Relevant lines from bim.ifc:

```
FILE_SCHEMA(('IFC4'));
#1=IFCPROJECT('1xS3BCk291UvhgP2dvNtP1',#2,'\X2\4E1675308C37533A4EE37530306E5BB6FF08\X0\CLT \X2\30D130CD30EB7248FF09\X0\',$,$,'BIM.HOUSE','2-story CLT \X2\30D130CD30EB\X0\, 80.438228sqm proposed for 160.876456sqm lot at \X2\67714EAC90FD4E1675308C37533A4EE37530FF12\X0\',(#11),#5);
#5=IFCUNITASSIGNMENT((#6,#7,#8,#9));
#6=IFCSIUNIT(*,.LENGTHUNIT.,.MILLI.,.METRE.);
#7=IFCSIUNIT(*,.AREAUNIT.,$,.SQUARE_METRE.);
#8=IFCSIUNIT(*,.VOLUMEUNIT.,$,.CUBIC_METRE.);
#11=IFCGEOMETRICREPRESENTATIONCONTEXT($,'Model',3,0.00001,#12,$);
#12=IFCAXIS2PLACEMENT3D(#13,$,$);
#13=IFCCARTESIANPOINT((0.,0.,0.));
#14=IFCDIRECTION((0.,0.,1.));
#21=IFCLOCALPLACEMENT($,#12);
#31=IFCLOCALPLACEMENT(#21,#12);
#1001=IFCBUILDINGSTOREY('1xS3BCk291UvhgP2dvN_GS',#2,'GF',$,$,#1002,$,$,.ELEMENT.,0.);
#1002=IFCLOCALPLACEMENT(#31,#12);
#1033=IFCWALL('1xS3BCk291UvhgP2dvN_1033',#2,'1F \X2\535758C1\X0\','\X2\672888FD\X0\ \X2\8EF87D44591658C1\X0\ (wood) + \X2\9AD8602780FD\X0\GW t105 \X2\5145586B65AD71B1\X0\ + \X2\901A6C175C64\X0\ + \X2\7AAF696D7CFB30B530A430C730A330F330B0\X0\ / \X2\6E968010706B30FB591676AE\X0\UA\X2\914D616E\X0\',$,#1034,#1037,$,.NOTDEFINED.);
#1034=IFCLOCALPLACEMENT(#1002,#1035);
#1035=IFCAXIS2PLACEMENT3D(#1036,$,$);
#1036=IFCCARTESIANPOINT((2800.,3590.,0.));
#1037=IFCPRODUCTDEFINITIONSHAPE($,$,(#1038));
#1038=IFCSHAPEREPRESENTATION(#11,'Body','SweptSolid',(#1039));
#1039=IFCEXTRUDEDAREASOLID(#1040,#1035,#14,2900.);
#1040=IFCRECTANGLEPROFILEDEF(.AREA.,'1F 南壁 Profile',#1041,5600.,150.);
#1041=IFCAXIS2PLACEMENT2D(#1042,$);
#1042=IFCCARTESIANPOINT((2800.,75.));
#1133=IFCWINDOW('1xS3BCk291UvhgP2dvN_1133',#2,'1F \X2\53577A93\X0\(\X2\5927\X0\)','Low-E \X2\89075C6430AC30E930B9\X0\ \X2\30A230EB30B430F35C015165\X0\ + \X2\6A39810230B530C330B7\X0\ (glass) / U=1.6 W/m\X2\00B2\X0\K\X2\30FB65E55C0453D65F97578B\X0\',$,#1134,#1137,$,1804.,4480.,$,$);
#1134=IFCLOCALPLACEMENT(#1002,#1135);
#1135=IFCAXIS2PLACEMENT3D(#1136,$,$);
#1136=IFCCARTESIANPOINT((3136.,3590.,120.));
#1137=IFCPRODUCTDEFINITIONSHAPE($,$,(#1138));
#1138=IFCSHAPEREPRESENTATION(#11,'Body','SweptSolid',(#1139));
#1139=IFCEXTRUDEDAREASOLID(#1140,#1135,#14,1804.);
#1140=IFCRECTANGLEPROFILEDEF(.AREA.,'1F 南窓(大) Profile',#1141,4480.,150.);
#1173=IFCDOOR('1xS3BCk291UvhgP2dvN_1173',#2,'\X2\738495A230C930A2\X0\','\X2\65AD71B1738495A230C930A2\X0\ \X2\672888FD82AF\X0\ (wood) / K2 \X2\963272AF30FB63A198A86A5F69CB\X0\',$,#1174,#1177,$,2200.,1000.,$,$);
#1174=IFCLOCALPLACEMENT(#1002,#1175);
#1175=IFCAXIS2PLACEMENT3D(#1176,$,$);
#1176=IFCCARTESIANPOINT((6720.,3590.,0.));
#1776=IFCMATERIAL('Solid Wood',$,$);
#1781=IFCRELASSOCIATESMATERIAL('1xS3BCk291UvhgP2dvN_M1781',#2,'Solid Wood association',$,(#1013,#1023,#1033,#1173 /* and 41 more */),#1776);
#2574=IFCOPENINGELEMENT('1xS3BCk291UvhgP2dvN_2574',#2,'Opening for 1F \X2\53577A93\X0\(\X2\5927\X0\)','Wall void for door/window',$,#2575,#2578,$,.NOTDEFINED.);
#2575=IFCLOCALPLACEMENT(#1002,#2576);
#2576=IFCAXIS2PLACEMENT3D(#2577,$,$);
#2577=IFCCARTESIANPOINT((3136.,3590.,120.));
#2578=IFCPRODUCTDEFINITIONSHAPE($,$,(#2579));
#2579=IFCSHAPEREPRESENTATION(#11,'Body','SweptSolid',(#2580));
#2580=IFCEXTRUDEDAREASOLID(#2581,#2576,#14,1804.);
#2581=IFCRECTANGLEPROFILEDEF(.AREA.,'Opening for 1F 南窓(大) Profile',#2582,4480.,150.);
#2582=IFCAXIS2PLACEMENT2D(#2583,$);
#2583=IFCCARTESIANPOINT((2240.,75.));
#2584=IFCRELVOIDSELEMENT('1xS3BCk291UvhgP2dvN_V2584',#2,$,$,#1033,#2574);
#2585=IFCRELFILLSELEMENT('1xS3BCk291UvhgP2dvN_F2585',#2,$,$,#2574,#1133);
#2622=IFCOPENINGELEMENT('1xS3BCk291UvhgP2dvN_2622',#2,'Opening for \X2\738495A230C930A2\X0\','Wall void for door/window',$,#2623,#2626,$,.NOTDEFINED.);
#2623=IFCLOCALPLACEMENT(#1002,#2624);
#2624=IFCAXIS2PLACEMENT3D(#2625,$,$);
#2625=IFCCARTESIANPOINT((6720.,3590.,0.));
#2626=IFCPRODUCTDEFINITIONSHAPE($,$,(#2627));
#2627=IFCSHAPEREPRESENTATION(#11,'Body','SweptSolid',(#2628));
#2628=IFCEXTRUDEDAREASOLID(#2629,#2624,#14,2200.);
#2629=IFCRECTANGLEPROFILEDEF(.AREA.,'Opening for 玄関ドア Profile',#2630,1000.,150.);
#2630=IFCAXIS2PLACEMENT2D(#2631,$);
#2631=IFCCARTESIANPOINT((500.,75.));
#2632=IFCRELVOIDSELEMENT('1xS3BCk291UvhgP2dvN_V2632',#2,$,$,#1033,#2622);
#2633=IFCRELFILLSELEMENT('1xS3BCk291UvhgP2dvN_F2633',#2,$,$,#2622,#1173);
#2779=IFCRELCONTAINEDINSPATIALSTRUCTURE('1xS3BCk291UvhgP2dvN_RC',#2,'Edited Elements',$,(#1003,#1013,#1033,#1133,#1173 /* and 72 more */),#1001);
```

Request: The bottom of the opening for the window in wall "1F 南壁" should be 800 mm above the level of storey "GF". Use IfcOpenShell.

```python
import numpy as np
import ifcopenshell
import ifcopenshell.api.geometry
import ifcopenshell.geom
import ifcopenshell.util.element
import ifcopenshell.util.placement
import ifcopenshell.util.shape
import ifcopenshell.util.unit

model = ifcopenshell.open("bim.ifc")
unit_scale = ifcopenshell.util.unit.calculate_unit_scale(model)

window = model.by_guid("1xS3BCk291UvhgP2dvN_1133")
opening = window.FillsVoids[0].RelatingOpeningElement
storey = ifcopenshell.util.element.get_container(window, ifc_class="IfcBuildingStorey")
level = ifcopenshell.util.placement.get_local_placement(storey.ObjectPlacement)[2, 3]

# The opening's origin need not be at the sill, so measure its lowest point.
shape = ifcopenshell.geom.create_shape(ifcopenshell.geom.settings(), opening)
bottom = ifcopenshell.util.shape.get_shape_bottom_elevation(shape, shape.geometry) / unit_scale
dz = level + 800.0 - bottom

shift = np.array([0.0, 0.0, dz])
# The window is not placed relative to its opening, so move both.
for product in (opening, window):
    matrix = ifcopenshell.util.placement.get_local_placement(product.ObjectPlacement)
    matrix[:3, 3] += shift
    ifcopenshell.api.geometry.edit_object_placement(model, product=product, matrix=matrix, is_si=False)

print(f"moved by {dz * unit_scale:+.3f} m")

model.write("bim-out.ifc")
```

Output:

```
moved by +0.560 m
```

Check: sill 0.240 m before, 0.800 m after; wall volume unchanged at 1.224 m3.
